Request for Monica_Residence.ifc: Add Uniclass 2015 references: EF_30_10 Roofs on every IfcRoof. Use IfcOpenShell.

First a look at what the model holds.

```python
import ifcopenshell

model = ifcopenshell.open("Monica_Residence.ifc")
print(model.schema)
print("classifications:", [c.Name for c in model.by_type("IfcClassification")])
for ifc_class in ("IfcDoor", "IfcRoof", "IfcStair", "IfcWall", "IfcWindow"):
    print(ifc_class, len(model.by_type(ifc_class)))
```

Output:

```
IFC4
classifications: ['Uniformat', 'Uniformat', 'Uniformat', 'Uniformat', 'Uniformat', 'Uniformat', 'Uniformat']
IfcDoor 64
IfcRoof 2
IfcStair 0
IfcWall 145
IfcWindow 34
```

```python
import ifcopenshell
import ifcopenshell.api.classification

model = ifcopenshell.open("Monica_Residence.ifc")

system = ifcopenshell.api.classification.add_classification(model, classification="Uniclass 2015")

codes = {
    "IfcRoof": ("EF_30_10", "Roofs"),
}
for ifc_class, (code, name) in codes.items():
    products = model.by_type(ifc_class)
    ifcopenshell.api.classification.add_reference(
        model, products=products, classification=system, identification=code, name=name
    )
    print(code, len(products))

model.write("Monica_Residence_rev.ifc")
```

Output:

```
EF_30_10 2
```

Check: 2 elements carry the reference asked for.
